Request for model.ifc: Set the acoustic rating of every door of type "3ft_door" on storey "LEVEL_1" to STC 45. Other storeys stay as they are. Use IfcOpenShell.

First a look at what the model holds.

```python
import ifcopenshell
import ifcopenshell.util.element

model = ifcopenshell.open("model.ifc")
print(model.schema)
storey = next(s for s in model.by_type("IfcBuildingStorey") if s.Name == "LEVEL_1")
doors = [e for e in ifcopenshell.util.element.get_decomposition(storey) if e.is_a("IfcDoor")]
seen = {}
for e in doors:
    element_type = ifcopenshell.util.element.get_type(e)
    key = (element_type.Name if element_type != e and element_type else None, ifcopenshell.util.element.get_pset(e, "Pset_DoorCommon", "AcousticRating"))
    seen[key] = seen.get(key, 0) + 1
for (name, value), count in sorted(seen.items(), key=str):
    print(count, "x", name, "|", value)
```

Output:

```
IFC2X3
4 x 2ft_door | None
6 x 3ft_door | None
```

```python
import ifcopenshell
import ifcopenshell.api.pset
import ifcopenshell.util.element

model = ifcopenshell.open("model.ifc")

storey = next(s for s in model.by_type("IfcBuildingStorey") if s.Name == "LEVEL_1")
doors = [e for e in ifcopenshell.util.element.get_decomposition(storey) if e.is_a("IfcDoor")]

count = 0
for e in doors:
    element_type = ifcopenshell.util.element.get_type(e)
    if element_type in (None, e) or element_type.Name != "3ft_door":
        continue
    # add_pset returns the element's existing set when there is one.
    pset = ifcopenshell.api.pset.add_pset(model, product=e, name="Pset_DoorCommon")
    ifcopenshell.api.pset.edit_pset(model, pset=pset, properties={"AcousticRating": "STC 45"})
    count += 1

print(count, "doors updated")

model.write("model-out.ifc")
```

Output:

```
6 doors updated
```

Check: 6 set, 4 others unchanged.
